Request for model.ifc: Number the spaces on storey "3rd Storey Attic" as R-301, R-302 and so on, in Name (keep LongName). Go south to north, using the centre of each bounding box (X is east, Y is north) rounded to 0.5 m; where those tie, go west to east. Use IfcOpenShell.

First a look at what the model holds.

```python
import ifcopenshell
import ifcopenshell.util.element
import ifcopenshell.util.placement

model = ifcopenshell.open("model.ifc")
print(model.schema)
storey = next(s for s in model.by_type("IfcBuildingStorey") if s.Name == "3rd Storey Attic")
spaces = [e for e in ifcopenshell.util.element.get_decomposition(storey) if e.is_a("IfcSpace")]
for e in sorted(spaces, key=lambda e: e.id()):
    origin = ifcopenshell.util.placement.get_local_placement(e.ObjectPlacement)[:3, 3]
    print(e.id(), e.Name, e.LongName, origin.round(2) + 0.0, sep=" | ")
```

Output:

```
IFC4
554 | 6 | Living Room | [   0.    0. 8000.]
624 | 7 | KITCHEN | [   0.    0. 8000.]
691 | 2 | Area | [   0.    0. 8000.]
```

```python
import ifcopenshell
import ifcopenshell.geom
import ifcopenshell.util.element
import ifcopenshell.util.shape

model = ifcopenshell.open("model.ifc")
settings = ifcopenshell.geom.settings()
settings.set("use-world-coords", True)


def centre(element):
    shape = ifcopenshell.geom.create_shape(settings, element)
    return ifcopenshell.util.shape.get_bbox_centroid(shape.geometry)


storey = next(s for s in model.by_type("IfcBuildingStorey") if s.Name == "3rd Storey Attic")
spaces = [e for e in ifcopenshell.util.element.get_decomposition(storey) if e.is_a("IfcSpace")]

# Insertion points can sit at a corner or the storey origin, so sort by the geometry (in metres).
centres = {e: centre(e) for e in spaces}
spaces.sort(key=lambda e: (round(centres[e][1] / 0.5), centres[e][0]))

for i, e in enumerate(spaces, start=1):
    number = f"R-3{i:02d}"
    e.Name = number
    print(e.id(), number)

model.write("model_updated.ifc")
```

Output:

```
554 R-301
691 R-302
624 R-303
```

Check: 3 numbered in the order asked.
